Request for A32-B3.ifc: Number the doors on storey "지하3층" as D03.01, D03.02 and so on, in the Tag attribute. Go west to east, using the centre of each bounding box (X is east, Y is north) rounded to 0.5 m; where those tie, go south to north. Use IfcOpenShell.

First a look at what the model holds.

```python
import ifcopenshell
import ifcopenshell.util.element
import ifcopenshell.util.placement

model = ifcopenshell.open("A32-B3.ifc")
print(model.schema)
storey = next(s for s in model.by_type("IfcBuildingStorey") if s.Name == "지하3층")
doors = [e for e in ifcopenshell.util.element.get_decomposition(storey) if e.is_a("IfcDoor")]
for e in sorted(doors, key=lambda e: e.id()):
    origin = ifcopenshell.util.placement.get_local_placement(e.ObjectPlacement)[:3, 3]
    print(e.id(), e.Tag, e.Name, origin.round(2) + 0.0, sep=" | ")
```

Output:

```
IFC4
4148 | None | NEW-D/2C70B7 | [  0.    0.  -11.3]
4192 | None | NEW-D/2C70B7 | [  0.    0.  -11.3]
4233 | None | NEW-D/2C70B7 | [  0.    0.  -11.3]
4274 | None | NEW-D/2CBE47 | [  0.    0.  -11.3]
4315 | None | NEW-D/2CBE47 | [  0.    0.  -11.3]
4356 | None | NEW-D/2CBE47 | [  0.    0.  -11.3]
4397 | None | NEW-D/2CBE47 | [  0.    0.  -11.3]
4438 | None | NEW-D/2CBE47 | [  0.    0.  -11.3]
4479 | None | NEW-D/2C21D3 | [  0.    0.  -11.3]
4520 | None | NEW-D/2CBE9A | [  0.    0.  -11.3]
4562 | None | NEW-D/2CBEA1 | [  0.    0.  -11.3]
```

```python
import ifcopenshell
import ifcopenshell.geom
import ifcopenshell.util.element
import ifcopenshell.util.shape

model = ifcopenshell.open("A32-B3.ifc")
settings = ifcopenshell.geom.settings()
settings.set("use-world-coords", True)


def centre(element):
    shape = ifcopenshell.geom.create_shape(settings, element)
    return ifcopenshell.util.shape.get_bbox_centroid(shape.geometry)


storey = next(s for s in model.by_type("IfcBuildingStorey") if s.Name == "지하3층")
doors = [e for e in ifcopenshell.util.element.get_decomposition(storey) if e.is_a("IfcDoor")]

# Insertion points can sit at a corner or the storey origin, so sort by the geometry (in metres).
centres = {e: centre(e) for e in doors}
doors.sort(key=lambda e: (round(centres[e][0] / 0.5), centres[e][1]))

for i, e in enumerate(doors, start=1):
    number = f"D03.{i:02d}"
    e.Tag = number
    print(e.id(), number)

model.write("A32-B3_v2.ifc")
```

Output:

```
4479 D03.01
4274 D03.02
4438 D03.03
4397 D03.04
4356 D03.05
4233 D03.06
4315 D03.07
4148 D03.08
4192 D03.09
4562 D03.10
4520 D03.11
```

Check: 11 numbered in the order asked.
